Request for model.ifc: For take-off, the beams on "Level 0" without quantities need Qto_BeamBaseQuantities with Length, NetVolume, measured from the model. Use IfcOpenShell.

First a look at what the model holds.

```python
import ifcopenshell
import ifcopenshell.util.element
import ifcopenshell.util.unit

model = ifcopenshell.open("model.ifc")
print(model.schema)
for unit_type in ("LENGTHUNIT", "AREAUNIT", "VOLUMEUNIT"):
    print(unit_type, ifcopenshell.util.unit.calculate_unit_scale(model, unit_type))
storey = next(s for s in model.by_type("IfcBuildingStorey") if s.Name == "Level 0")
beams = [e for e in ifcopenshell.util.element.get_decomposition(storey) if e.is_a("IfcBeam")]
for e in sorted(beams, key=lambda e: e.id()):
    print(e.id(), e.is_a(), e.Name, list(ifcopenshell.util.element.get_psets(e, qtos_only=True)), sep=" | ")
```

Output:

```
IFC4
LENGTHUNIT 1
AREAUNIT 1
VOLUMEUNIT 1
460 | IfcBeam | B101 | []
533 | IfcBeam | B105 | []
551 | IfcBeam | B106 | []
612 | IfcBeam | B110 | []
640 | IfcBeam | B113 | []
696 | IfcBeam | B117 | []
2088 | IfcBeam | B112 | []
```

```python
import ifcopenshell
import ifcopenshell.api.pset
import ifcopenshell.geom
import ifcopenshell.util.element
import ifcopenshell.util.shape
import ifcopenshell.util.unit

model = ifcopenshell.open("model.ifc")
unit_scale = ifcopenshell.util.unit.calculate_unit_scale(model)
volume_scale = ifcopenshell.util.unit.calculate_unit_scale(model, "VOLUMEUNIT")
settings = ifcopenshell.geom.settings()

storey = next(s for s in model.by_type("IfcBuildingStorey") if s.Name == "Level 0")
beams = [e for e in ifcopenshell.util.element.get_decomposition(storey) if e.is_a("IfcBeam")]

for e in sorted(beams, key=lambda e: e.id()):
    if ifcopenshell.util.element.get_psets(e, qtos_only=True, should_inherit=False):
        continue
    # Geometry comes back in metres, in the element's own axes.
    shape = ifcopenshell.geom.create_shape(settings, e)
    values = {
        "Length": ifcopenshell.util.shape.get_max_xyz(shape.geometry) / unit_scale,
        "NetVolume": ifcopenshell.util.shape.get_volume(shape.geometry) / volume_scale,
    }
    qto = ifcopenshell.api.pset.add_qto(model, product=e, name="Qto_BeamBaseQuantities")
    ifcopenshell.api.pset.edit_qto(model, qto=qto, properties=values)
    print(e.id(), {k: round(v, 3) for k, v in values.items()})

model.write("model_edited.ifc")
```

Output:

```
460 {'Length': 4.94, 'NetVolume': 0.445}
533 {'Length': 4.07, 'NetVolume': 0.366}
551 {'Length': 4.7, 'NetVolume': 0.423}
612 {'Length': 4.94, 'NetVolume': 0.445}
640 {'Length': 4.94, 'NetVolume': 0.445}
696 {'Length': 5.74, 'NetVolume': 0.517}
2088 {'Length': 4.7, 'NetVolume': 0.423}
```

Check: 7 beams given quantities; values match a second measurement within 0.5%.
